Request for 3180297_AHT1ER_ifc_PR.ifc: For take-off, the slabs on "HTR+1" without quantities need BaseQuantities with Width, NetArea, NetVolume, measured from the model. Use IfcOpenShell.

First a look at what the model holds.

```python
import ifcopenshell
import ifcopenshell.util.element
import ifcopenshell.util.unit

model = ifcopenshell.open("3180297_AHT1ER_ifc_PR.ifc")
print(model.schema)
for unit_type in ("LENGTHUNIT", "AREAUNIT", "VOLUMEUNIT"):
    print(unit_type, ifcopenshell.util.unit.calculate_unit_scale(model, unit_type))
storey = next(s for s in model.by_type("IfcBuildingStorey") if s.Name == "HTR+1")
slabs = [e for e in ifcopenshell.util.element.get_decomposition(storey) if e.is_a("IfcSlab")]
for e in sorted(slabs, key=lambda e: e.id()):
    print(e.id(), e.is_a(), e.Name, list(ifcopenshell.util.element.get_psets(e, qtos_only=True)), sep=" | ")
```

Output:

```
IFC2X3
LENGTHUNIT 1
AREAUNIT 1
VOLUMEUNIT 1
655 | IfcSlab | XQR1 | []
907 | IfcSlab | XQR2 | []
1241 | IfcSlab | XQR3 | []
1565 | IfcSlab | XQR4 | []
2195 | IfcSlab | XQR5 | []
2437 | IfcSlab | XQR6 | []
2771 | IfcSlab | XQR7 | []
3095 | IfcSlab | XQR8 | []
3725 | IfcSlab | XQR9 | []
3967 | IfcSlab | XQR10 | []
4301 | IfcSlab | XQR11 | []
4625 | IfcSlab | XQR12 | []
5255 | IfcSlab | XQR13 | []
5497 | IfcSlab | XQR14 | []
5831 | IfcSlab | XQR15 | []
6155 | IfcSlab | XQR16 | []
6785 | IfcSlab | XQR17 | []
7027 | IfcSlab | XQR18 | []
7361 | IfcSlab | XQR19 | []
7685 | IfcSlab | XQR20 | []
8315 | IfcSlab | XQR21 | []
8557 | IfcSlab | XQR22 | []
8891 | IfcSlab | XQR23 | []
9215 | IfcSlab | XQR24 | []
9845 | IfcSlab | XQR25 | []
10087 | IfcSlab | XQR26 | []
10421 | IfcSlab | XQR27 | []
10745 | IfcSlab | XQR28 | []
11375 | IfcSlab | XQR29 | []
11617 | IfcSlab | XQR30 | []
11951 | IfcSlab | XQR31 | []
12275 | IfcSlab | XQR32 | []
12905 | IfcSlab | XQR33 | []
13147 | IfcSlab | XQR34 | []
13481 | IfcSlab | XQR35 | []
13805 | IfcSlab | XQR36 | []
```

```python
import ifcopenshell
import ifcopenshell.api.pset
import ifcopenshell.geom
import ifcopenshell.util.element
import ifcopenshell.util.shape
import ifcopenshell.util.unit

model = ifcopenshell.open("3180297_AHT1ER_ifc_PR.ifc")
unit_scale = ifcopenshell.util.unit.calculate_unit_scale(model)
area_scale = ifcopenshell.util.unit.calculate_unit_scale(model, "AREAUNIT")
volume_scale = ifcopenshell.util.unit.calculate_unit_scale(model, "VOLUMEUNIT")
settings = ifcopenshell.geom.settings()

storey = next(s for s in model.by_type("IfcBuildingStorey") if s.Name == "HTR+1")
slabs = [e for e in ifcopenshell.util.element.get_decomposition(storey) if e.is_a("IfcSlab")]

for e in sorted(slabs, key=lambda e: e.id()):
    if ifcopenshell.util.element.get_psets(e, qtos_only=True, should_inherit=False):
        continue
    # Geometry comes back in metres, in the element's own axes.
    shape = ifcopenshell.geom.create_shape(settings, e)
    values = {
        "Width": ifcopenshell.util.shape.get_z(shape.geometry) / unit_scale,
        "NetArea": ifcopenshell.util.shape.get_footprint_area(shape.geometry) / area_scale,
        "NetVolume": ifcopenshell.util.shape.get_volume(shape.geometry) / volume_scale,
    }
    qto = ifcopenshell.api.pset.add_qto(model, product=e, name="BaseQuantities")
    ifcopenshell.api.pset.edit_qto(model, qto=qto, properties=values)
    print(e.id(), {k: round(v, 3) for k, v in values.items()})

model.write("3180297_AHT1ER_ifc_PR-out.ifc")
```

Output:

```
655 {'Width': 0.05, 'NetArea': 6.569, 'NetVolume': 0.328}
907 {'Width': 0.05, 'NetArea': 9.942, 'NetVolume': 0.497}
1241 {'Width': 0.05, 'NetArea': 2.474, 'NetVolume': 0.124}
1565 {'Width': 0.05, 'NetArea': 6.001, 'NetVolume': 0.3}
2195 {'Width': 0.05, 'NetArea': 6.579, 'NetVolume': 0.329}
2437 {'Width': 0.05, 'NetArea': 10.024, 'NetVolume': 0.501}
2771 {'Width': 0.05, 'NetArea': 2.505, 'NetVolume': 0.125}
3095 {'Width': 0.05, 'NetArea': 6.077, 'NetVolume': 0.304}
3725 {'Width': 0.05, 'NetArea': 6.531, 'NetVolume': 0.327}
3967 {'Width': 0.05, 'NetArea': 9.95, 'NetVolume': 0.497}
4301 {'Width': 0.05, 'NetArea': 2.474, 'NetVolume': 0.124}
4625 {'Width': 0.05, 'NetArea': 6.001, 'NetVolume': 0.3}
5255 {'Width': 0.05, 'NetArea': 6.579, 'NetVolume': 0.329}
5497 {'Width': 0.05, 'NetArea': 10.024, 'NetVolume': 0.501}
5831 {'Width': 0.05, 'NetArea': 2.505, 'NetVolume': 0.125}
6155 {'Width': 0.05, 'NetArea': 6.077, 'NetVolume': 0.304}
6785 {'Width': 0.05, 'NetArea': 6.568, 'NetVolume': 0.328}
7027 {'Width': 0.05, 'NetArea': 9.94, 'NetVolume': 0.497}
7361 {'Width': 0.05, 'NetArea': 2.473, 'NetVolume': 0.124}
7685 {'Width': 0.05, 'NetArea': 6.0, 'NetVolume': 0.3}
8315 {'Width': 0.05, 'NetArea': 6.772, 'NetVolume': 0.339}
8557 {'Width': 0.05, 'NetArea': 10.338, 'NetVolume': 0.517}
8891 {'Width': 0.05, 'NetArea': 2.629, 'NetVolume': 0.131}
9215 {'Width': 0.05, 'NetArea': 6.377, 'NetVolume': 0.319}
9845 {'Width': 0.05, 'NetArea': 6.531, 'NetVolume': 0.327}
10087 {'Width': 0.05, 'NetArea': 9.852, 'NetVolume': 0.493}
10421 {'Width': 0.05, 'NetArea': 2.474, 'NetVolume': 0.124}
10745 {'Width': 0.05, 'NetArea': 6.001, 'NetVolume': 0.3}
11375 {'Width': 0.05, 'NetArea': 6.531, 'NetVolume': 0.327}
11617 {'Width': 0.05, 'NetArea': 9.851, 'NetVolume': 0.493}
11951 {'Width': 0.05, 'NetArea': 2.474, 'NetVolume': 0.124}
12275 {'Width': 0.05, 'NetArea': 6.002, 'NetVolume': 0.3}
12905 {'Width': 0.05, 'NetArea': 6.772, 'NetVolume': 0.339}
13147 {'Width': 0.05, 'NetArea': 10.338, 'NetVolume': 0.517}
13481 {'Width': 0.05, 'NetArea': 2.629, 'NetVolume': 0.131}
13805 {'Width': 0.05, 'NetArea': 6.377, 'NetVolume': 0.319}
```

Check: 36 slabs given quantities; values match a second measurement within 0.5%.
